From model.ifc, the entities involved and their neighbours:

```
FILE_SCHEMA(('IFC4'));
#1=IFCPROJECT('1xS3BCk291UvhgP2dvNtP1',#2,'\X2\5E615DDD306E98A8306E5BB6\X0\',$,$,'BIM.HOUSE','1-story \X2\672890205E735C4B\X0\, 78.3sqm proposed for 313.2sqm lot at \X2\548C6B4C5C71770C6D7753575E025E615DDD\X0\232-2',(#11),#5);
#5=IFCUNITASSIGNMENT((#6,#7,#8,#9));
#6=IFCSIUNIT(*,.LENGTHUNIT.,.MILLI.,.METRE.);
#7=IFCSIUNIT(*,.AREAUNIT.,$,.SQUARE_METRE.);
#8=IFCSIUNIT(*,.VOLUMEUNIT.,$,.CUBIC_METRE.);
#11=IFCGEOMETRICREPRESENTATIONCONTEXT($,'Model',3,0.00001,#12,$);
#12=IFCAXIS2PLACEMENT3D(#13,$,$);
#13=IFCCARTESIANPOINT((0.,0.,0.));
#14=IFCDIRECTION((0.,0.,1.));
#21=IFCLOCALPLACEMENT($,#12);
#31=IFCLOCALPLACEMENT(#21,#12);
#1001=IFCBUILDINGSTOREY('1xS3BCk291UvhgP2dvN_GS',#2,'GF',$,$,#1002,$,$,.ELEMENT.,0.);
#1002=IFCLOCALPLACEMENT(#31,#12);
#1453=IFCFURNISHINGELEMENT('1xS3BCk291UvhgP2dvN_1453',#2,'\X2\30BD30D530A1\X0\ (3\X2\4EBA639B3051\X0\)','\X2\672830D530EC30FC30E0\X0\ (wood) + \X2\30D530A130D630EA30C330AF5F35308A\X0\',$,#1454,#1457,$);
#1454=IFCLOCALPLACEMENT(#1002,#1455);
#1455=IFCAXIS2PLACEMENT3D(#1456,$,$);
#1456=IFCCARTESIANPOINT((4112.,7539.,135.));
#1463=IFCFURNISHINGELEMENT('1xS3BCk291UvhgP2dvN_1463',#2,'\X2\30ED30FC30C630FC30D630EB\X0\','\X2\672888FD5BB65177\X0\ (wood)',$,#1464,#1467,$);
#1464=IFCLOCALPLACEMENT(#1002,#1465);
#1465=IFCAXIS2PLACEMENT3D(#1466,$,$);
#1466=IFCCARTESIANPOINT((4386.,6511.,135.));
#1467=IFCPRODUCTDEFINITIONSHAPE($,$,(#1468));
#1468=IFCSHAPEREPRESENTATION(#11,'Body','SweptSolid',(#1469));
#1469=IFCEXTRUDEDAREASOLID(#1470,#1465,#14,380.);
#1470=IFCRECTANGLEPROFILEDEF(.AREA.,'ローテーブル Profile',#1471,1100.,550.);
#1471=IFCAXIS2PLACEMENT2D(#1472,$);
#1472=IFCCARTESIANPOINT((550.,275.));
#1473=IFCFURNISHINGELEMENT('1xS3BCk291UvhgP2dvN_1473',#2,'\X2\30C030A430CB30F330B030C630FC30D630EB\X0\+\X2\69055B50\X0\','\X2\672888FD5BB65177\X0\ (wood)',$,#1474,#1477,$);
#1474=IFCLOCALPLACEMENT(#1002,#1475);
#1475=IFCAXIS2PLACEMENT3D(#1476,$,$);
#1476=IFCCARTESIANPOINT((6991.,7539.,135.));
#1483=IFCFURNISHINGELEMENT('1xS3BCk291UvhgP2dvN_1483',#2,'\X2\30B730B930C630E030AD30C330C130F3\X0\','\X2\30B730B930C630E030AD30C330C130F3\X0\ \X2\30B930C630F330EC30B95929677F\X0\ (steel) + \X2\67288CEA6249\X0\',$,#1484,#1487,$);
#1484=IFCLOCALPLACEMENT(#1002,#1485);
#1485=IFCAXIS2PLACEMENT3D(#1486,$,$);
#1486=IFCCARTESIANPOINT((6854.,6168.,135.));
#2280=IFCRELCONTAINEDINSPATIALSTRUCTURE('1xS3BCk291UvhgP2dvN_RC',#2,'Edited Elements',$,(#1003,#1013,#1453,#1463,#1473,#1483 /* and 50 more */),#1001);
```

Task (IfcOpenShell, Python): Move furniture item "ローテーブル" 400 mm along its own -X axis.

```python
import ifcopenshell
import ifcopenshell.api.geometry
import ifcopenshell.util.placement
import ifcopenshell.util.unit

model = ifcopenshell.open("model.ifc")
unit_scale = ifcopenshell.util.unit.calculate_unit_scale(model)

item = model.by_guid("1xS3BCk291UvhgP2dvN_1463")
matrix = ifcopenshell.util.placement.get_local_placement(item.ObjectPlacement)
matrix[:3, 3] -= matrix[:3, 0] * 0.4 / unit_scale
ifcopenshell.api.geometry.edit_object_placement(model, product=item, matrix=matrix, is_si=False)

print(ifcopenshell.util.placement.get_local_placement(item.ObjectPlacement).round(3) + 0.0)

model.write("model-out.ifc")
```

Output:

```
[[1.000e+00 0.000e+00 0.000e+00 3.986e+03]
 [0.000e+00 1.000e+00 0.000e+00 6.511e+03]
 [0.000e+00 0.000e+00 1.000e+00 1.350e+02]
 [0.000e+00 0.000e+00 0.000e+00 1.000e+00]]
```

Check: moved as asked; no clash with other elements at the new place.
